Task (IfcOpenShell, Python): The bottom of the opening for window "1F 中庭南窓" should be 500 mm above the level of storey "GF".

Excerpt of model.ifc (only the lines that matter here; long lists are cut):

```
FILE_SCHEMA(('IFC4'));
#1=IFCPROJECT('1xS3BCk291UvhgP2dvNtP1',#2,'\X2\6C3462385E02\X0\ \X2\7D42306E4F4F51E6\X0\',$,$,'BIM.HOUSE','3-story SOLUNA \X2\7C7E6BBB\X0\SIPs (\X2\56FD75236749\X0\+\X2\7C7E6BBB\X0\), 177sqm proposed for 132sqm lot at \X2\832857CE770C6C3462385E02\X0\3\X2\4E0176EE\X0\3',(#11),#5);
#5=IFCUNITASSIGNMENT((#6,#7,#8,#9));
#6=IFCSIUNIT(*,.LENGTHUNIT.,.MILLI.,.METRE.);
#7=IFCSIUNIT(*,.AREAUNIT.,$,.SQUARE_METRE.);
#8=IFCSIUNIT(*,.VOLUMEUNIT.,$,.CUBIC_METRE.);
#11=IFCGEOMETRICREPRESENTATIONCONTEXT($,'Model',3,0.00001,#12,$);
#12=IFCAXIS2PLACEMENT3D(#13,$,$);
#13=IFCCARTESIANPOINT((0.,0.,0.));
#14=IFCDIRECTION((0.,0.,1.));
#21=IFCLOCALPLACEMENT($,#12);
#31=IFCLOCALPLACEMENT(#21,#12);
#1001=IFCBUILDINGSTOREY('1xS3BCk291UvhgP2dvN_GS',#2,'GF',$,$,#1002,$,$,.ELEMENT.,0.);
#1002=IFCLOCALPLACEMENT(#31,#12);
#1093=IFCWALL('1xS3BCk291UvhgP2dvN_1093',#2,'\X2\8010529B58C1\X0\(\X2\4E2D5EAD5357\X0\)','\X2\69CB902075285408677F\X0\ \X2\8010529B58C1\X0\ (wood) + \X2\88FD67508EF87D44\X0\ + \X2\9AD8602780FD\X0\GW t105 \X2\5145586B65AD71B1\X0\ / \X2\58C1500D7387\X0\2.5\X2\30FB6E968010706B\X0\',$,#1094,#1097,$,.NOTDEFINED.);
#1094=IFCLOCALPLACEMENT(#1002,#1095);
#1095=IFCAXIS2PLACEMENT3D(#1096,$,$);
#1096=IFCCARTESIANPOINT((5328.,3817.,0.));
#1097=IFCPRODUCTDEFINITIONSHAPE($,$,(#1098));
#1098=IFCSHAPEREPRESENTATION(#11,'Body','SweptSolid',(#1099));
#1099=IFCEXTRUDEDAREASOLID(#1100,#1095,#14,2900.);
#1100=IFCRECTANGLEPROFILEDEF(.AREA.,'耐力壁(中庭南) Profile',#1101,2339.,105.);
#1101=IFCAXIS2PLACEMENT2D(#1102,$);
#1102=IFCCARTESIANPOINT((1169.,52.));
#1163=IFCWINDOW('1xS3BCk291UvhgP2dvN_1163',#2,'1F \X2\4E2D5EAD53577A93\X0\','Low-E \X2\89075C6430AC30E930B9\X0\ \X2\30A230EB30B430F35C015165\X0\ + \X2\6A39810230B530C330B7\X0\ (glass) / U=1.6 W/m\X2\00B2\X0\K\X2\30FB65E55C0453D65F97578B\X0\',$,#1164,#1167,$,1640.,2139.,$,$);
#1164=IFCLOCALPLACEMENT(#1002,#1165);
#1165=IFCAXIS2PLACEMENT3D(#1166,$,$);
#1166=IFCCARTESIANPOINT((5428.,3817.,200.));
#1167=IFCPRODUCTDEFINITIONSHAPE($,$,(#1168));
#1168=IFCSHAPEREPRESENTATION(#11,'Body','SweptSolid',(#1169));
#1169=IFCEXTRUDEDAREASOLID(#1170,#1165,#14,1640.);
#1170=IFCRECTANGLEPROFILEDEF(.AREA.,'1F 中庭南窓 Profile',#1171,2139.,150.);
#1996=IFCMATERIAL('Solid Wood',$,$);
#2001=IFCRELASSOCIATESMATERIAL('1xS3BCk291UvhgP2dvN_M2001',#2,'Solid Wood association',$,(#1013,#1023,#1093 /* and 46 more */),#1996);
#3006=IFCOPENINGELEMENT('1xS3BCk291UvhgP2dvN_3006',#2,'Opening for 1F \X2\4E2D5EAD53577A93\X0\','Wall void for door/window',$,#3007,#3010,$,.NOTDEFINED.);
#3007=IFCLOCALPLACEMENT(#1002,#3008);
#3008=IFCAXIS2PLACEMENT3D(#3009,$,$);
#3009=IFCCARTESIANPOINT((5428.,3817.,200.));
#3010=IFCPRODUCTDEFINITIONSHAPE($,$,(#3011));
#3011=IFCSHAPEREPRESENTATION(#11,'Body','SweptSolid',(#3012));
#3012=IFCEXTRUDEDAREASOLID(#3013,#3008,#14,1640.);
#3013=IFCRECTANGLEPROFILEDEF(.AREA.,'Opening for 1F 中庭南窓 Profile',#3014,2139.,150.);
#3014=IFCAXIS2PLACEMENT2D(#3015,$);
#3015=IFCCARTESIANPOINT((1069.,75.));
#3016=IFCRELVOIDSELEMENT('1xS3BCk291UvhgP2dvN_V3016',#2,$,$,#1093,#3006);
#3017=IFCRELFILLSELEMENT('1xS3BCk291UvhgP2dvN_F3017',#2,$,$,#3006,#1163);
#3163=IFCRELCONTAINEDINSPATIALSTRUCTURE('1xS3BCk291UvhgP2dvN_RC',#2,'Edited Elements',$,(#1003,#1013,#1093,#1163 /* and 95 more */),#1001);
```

```python
import numpy as np
import ifcopenshell
import ifcopenshell.api.geometry
import ifcopenshell.geom
import ifcopenshell.util.element
import ifcopenshell.util.placement
import ifcopenshell.util.shape
import ifcopenshell.util.unit

model = ifcopenshell.open("model.ifc")
unit_scale = ifcopenshell.util.unit.calculate_unit_scale(model)

window = model.by_guid("1xS3BCk291UvhgP2dvN_1163")
opening = window.FillsVoids[0].RelatingOpeningElement
storey = ifcopenshell.util.element.get_container(window, ifc_class="IfcBuildingStorey")
level = ifcopenshell.util.placement.get_local_placement(storey.ObjectPlacement)[2, 3]

# The opening's origin need not be at the sill, so measure its lowest point.
shape = ifcopenshell.geom.create_shape(ifcopenshell.geom.settings(), opening)
bottom = ifcopenshell.util.shape.get_shape_bottom_elevation(shape, shape.geometry) / unit_scale
dz = level + 500.0 - bottom

shift = np.array([0.0, 0.0, dz])
# The window is not placed relative to its opening, so move both.
for product in (opening, window):
    matrix = ifcopenshell.util.placement.get_local_placement(product.ObjectPlacement)
    matrix[:3, 3] += shift
    ifcopenshell.api.geometry.edit_object_placement(model, product=product, matrix=matrix, is_si=False)

print(f"moved by {dz * unit_scale:+.3f} m")

model.write("model_updated.ifc")
```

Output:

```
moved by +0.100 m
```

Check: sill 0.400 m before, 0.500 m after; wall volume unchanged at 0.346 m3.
